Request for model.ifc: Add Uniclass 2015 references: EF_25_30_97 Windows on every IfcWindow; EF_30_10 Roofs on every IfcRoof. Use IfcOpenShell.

First a look at what the model holds.

```python
import ifcopenshell

model = ifcopenshell.open("model.ifc")
print(model.schema)
print("classifications:", [c.Name for c in model.by_type("IfcClassification")])
for ifc_class in ("IfcDoor", "IfcRoof", "IfcStair", "IfcWall", "IfcWindow"):
    print(ifc_class, len(model.by_type(ifc_class)))
```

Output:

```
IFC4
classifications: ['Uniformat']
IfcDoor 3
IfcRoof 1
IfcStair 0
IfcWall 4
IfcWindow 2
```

```python
import ifcopenshell
import ifcopenshell.api.classification

model = ifcopenshell.open("model.ifc")

system = ifcopenshell.api.classification.add_classification(model, classification="Uniclass 2015")

codes = {
    "IfcWindow": ("EF_25_30_97", "Windows"),
    "IfcRoof": ("EF_30_10", "Roofs"),
}
for ifc_class, (code, name) in codes.items():
    products = model.by_type(ifc_class)
    ifcopenshell.api.classification.add_reference(
        model, products=products, classification=system, identification=code, name=name
    )
    print(code, len(products))

model.write("model_rev.ifc")
```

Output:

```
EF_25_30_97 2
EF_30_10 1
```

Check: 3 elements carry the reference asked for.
